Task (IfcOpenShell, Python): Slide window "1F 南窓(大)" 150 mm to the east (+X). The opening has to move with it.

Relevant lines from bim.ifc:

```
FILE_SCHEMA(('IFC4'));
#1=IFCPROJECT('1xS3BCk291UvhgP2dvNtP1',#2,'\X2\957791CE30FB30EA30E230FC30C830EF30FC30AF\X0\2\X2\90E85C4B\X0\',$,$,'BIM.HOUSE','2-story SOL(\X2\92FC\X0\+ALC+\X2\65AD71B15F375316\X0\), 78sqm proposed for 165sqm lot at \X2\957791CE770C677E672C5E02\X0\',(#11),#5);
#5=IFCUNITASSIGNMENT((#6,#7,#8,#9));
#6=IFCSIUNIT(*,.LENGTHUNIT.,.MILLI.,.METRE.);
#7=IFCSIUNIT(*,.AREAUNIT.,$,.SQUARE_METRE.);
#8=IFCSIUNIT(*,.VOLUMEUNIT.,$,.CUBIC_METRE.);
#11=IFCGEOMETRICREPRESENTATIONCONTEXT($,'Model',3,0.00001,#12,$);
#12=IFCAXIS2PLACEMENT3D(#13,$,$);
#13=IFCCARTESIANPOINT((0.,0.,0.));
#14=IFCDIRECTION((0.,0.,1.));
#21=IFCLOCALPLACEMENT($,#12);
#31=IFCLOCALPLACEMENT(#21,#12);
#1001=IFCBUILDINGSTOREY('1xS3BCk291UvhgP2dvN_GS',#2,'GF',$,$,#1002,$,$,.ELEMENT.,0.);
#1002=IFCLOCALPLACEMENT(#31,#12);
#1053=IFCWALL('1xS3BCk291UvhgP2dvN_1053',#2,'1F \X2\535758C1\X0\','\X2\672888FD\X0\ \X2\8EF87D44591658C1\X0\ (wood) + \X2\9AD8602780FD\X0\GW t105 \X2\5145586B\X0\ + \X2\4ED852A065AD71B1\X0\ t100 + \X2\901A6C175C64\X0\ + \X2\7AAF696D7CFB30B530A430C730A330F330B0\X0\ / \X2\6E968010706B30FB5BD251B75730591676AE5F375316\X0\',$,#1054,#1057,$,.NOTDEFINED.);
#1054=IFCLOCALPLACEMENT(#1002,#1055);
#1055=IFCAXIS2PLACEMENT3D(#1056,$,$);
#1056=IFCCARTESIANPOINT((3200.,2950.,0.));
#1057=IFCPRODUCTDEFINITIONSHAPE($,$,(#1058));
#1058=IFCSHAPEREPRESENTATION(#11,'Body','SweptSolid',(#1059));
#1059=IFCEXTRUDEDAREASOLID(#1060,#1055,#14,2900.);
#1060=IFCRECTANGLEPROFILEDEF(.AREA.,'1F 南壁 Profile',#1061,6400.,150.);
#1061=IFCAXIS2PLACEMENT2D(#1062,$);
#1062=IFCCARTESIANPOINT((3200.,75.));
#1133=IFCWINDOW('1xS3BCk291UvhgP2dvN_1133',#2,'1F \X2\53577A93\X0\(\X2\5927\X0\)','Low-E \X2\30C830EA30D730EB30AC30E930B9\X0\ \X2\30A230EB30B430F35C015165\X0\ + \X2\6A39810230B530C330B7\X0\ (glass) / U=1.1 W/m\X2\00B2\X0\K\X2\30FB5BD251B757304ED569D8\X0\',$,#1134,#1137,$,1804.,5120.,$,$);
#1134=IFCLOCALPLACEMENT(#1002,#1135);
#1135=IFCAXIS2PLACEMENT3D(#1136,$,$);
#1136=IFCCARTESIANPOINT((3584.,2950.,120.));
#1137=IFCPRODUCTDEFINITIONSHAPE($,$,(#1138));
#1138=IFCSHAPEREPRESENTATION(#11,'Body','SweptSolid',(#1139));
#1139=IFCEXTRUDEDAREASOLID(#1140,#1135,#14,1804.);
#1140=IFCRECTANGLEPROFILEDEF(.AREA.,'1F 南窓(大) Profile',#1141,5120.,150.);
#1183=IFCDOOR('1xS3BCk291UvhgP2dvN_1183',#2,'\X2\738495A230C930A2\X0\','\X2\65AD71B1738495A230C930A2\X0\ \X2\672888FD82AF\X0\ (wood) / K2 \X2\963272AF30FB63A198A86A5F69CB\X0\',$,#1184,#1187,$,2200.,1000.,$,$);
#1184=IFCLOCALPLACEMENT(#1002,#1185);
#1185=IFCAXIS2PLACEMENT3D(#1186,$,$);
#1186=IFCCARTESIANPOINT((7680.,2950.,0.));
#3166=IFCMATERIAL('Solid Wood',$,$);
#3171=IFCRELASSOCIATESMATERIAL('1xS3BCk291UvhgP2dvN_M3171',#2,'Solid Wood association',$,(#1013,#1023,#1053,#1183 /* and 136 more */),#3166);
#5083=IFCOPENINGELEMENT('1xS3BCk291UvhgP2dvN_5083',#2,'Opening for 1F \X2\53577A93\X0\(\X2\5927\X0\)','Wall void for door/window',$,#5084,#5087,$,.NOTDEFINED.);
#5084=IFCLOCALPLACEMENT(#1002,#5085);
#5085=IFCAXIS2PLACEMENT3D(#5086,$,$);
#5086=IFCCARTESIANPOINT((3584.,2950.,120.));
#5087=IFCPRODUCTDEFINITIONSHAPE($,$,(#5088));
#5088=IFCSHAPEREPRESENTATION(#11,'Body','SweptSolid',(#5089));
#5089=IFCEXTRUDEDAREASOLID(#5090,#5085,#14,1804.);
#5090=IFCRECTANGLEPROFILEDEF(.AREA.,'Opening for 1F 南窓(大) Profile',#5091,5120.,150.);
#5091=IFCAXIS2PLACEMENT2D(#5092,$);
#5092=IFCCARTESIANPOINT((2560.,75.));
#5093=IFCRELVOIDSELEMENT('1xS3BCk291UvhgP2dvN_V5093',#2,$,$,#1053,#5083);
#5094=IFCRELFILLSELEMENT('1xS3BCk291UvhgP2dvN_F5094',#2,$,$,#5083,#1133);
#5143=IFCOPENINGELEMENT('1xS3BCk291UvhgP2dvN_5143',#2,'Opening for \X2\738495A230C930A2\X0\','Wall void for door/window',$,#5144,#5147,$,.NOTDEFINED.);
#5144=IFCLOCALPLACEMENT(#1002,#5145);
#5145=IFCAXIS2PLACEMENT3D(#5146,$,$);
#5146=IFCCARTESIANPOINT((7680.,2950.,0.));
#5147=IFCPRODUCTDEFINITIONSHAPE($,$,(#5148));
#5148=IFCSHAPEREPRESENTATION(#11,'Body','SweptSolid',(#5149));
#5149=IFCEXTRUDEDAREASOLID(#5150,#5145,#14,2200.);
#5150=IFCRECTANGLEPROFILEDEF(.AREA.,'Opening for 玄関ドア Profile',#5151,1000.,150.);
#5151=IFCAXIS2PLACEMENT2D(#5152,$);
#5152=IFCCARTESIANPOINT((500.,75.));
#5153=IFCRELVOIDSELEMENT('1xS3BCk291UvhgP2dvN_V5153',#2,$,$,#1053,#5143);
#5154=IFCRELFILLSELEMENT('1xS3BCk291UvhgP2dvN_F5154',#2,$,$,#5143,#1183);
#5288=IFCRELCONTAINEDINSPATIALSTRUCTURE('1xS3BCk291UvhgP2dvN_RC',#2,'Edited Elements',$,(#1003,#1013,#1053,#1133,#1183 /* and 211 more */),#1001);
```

```python
import ifcopenshell
import ifcopenshell.api.geometry
import ifcopenshell.util.placement
import ifcopenshell.util.unit

model = ifcopenshell.open("bim.ifc")
unit_scale = ifcopenshell.util.unit.calculate_unit_scale(model)

window = model.by_id(1133)
opening = window.FillsVoids[0].RelatingOpeningElement
wall = opening.VoidsElements[0].RelatingBuildingElement

wall_matrix = ifcopenshell.util.placement.get_local_placement(wall.ObjectPlacement)
shift = wall_matrix[:3, 0] * 0.15 / unit_scale
before = ifcopenshell.util.placement.get_local_placement(window.ObjectPlacement)[:3, 3].copy()

# The window is not placed relative to its opening, so move both.
for product in (opening, window):
    matrix = ifcopenshell.util.placement.get_local_placement(product.ObjectPlacement)
    matrix[:3, 3] += shift
    ifcopenshell.api.geometry.edit_object_placement(model, product=product, matrix=matrix, is_si=False)

after = ifcopenshell.util.placement.get_local_placement(window.ObjectPlacement)[:3, 3]
print("window moved by", (after - before).round(3) + 0.0)

model.write("bim-out.ifc")
```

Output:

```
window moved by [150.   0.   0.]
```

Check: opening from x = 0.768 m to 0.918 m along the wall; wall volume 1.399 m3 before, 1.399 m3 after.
